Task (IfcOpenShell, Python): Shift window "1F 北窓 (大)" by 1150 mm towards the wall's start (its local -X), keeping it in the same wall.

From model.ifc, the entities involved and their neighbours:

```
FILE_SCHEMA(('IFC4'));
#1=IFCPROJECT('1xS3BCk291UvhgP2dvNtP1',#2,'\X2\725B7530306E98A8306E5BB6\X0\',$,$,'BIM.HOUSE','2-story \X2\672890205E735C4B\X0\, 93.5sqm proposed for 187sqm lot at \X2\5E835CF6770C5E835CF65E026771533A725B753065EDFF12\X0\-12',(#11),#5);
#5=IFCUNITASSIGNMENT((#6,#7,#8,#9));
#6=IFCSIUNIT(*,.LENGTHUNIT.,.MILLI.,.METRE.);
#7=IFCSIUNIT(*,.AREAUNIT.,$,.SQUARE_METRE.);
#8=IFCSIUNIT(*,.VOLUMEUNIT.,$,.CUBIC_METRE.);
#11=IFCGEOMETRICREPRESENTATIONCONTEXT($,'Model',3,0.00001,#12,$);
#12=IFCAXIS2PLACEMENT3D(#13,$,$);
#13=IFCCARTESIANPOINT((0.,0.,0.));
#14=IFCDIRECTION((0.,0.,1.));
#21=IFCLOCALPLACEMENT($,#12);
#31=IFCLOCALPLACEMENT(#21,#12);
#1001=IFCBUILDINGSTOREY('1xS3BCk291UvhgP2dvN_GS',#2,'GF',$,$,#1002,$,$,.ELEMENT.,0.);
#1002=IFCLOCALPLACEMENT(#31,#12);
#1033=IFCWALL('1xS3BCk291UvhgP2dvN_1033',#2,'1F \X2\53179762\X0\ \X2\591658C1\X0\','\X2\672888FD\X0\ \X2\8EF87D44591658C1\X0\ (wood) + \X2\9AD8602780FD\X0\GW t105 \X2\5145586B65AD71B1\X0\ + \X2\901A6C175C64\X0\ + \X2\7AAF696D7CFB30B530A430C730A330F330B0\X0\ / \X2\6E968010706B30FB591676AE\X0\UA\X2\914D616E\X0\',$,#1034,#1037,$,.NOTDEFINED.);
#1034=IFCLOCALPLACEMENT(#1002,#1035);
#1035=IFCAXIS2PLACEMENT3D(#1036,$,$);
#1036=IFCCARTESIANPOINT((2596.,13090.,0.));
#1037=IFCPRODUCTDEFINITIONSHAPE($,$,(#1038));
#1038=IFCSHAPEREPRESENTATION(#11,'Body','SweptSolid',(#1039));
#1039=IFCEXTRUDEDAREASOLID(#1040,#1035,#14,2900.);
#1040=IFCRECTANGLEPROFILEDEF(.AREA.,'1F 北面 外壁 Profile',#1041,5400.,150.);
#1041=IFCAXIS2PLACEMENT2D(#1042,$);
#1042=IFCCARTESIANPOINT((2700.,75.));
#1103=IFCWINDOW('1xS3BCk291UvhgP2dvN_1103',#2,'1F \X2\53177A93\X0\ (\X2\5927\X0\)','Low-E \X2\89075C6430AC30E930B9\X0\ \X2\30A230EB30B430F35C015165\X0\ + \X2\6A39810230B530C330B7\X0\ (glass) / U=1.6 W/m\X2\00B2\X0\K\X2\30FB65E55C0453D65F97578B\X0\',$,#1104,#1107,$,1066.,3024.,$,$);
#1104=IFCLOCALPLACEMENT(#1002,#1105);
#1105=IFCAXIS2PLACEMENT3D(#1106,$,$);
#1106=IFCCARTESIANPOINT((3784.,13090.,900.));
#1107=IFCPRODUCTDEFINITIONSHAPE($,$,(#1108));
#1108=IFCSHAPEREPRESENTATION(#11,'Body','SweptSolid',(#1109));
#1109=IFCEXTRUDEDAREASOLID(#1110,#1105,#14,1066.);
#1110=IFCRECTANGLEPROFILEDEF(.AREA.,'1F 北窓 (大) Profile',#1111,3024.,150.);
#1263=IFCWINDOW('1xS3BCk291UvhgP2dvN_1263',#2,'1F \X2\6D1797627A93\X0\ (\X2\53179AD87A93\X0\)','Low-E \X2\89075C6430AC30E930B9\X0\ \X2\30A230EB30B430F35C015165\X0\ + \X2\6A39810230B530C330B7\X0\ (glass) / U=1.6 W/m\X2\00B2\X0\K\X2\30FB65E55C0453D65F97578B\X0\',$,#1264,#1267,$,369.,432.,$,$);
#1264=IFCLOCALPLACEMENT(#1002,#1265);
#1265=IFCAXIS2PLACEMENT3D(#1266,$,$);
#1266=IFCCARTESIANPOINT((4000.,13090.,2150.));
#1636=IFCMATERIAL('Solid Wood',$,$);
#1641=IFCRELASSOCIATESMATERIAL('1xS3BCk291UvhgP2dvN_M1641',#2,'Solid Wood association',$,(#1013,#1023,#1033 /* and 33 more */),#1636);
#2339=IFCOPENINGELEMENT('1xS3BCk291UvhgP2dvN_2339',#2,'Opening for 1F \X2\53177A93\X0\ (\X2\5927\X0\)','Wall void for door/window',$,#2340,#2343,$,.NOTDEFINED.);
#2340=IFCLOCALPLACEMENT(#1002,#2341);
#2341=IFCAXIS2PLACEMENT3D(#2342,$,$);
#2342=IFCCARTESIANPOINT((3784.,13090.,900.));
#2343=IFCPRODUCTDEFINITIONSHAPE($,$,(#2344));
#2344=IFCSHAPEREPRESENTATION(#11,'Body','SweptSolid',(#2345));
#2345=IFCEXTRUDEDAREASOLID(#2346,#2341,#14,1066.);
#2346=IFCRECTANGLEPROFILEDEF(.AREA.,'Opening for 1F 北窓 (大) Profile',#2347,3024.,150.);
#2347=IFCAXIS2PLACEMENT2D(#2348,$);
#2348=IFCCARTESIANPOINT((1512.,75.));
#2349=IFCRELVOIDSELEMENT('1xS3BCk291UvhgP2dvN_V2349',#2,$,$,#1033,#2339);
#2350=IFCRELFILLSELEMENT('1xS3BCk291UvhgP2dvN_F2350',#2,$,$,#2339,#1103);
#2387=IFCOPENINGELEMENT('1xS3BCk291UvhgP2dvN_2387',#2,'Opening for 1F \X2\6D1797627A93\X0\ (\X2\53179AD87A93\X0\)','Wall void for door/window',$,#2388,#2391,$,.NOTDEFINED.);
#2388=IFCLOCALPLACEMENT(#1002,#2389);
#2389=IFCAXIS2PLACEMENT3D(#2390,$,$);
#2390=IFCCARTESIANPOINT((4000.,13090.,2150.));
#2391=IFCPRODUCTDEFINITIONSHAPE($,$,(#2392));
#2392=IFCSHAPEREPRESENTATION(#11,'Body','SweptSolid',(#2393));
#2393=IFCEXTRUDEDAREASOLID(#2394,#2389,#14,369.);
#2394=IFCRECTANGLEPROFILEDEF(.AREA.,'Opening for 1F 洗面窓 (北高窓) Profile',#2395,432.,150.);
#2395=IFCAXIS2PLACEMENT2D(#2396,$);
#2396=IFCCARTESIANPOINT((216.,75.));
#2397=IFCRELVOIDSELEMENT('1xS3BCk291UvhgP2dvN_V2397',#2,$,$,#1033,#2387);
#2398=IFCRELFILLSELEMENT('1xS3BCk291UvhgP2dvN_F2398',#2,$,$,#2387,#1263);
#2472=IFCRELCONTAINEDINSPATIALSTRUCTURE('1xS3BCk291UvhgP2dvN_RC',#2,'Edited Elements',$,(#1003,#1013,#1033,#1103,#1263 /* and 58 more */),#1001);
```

```python
import ifcopenshell
import ifcopenshell.api.geometry
import ifcopenshell.util.placement
import ifcopenshell.util.unit

model = ifcopenshell.open("model.ifc")
unit_scale = ifcopenshell.util.unit.calculate_unit_scale(model)

window = model.by_guid("1xS3BCk291UvhgP2dvN_1103")
opening = window.FillsVoids[0].RelatingOpeningElement
wall = opening.VoidsElements[0].RelatingBuildingElement

wall_matrix = ifcopenshell.util.placement.get_local_placement(wall.ObjectPlacement)
shift = wall_matrix[:3, 0] * -1.15 / unit_scale
before = ifcopenshell.util.placement.get_local_placement(window.ObjectPlacement)[:3, 3].copy()

# The window is not placed relative to its opening, so move both.
for product in (opening, window):
    matrix = ifcopenshell.util.placement.get_local_placement(product.ObjectPlacement)
    matrix[:3, 3] += shift
    ifcopenshell.api.geometry.edit_object_placement(model, product=product, matrix=matrix, is_si=False)

after = ifcopenshell.util.placement.get_local_placement(window.ObjectPlacement)[:3, 3]
print("window moved by", (after - before).round(3) + 0.0)

model.write("model_rev.ifc")
```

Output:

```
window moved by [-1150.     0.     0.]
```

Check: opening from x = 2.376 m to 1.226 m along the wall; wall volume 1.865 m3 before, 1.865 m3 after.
